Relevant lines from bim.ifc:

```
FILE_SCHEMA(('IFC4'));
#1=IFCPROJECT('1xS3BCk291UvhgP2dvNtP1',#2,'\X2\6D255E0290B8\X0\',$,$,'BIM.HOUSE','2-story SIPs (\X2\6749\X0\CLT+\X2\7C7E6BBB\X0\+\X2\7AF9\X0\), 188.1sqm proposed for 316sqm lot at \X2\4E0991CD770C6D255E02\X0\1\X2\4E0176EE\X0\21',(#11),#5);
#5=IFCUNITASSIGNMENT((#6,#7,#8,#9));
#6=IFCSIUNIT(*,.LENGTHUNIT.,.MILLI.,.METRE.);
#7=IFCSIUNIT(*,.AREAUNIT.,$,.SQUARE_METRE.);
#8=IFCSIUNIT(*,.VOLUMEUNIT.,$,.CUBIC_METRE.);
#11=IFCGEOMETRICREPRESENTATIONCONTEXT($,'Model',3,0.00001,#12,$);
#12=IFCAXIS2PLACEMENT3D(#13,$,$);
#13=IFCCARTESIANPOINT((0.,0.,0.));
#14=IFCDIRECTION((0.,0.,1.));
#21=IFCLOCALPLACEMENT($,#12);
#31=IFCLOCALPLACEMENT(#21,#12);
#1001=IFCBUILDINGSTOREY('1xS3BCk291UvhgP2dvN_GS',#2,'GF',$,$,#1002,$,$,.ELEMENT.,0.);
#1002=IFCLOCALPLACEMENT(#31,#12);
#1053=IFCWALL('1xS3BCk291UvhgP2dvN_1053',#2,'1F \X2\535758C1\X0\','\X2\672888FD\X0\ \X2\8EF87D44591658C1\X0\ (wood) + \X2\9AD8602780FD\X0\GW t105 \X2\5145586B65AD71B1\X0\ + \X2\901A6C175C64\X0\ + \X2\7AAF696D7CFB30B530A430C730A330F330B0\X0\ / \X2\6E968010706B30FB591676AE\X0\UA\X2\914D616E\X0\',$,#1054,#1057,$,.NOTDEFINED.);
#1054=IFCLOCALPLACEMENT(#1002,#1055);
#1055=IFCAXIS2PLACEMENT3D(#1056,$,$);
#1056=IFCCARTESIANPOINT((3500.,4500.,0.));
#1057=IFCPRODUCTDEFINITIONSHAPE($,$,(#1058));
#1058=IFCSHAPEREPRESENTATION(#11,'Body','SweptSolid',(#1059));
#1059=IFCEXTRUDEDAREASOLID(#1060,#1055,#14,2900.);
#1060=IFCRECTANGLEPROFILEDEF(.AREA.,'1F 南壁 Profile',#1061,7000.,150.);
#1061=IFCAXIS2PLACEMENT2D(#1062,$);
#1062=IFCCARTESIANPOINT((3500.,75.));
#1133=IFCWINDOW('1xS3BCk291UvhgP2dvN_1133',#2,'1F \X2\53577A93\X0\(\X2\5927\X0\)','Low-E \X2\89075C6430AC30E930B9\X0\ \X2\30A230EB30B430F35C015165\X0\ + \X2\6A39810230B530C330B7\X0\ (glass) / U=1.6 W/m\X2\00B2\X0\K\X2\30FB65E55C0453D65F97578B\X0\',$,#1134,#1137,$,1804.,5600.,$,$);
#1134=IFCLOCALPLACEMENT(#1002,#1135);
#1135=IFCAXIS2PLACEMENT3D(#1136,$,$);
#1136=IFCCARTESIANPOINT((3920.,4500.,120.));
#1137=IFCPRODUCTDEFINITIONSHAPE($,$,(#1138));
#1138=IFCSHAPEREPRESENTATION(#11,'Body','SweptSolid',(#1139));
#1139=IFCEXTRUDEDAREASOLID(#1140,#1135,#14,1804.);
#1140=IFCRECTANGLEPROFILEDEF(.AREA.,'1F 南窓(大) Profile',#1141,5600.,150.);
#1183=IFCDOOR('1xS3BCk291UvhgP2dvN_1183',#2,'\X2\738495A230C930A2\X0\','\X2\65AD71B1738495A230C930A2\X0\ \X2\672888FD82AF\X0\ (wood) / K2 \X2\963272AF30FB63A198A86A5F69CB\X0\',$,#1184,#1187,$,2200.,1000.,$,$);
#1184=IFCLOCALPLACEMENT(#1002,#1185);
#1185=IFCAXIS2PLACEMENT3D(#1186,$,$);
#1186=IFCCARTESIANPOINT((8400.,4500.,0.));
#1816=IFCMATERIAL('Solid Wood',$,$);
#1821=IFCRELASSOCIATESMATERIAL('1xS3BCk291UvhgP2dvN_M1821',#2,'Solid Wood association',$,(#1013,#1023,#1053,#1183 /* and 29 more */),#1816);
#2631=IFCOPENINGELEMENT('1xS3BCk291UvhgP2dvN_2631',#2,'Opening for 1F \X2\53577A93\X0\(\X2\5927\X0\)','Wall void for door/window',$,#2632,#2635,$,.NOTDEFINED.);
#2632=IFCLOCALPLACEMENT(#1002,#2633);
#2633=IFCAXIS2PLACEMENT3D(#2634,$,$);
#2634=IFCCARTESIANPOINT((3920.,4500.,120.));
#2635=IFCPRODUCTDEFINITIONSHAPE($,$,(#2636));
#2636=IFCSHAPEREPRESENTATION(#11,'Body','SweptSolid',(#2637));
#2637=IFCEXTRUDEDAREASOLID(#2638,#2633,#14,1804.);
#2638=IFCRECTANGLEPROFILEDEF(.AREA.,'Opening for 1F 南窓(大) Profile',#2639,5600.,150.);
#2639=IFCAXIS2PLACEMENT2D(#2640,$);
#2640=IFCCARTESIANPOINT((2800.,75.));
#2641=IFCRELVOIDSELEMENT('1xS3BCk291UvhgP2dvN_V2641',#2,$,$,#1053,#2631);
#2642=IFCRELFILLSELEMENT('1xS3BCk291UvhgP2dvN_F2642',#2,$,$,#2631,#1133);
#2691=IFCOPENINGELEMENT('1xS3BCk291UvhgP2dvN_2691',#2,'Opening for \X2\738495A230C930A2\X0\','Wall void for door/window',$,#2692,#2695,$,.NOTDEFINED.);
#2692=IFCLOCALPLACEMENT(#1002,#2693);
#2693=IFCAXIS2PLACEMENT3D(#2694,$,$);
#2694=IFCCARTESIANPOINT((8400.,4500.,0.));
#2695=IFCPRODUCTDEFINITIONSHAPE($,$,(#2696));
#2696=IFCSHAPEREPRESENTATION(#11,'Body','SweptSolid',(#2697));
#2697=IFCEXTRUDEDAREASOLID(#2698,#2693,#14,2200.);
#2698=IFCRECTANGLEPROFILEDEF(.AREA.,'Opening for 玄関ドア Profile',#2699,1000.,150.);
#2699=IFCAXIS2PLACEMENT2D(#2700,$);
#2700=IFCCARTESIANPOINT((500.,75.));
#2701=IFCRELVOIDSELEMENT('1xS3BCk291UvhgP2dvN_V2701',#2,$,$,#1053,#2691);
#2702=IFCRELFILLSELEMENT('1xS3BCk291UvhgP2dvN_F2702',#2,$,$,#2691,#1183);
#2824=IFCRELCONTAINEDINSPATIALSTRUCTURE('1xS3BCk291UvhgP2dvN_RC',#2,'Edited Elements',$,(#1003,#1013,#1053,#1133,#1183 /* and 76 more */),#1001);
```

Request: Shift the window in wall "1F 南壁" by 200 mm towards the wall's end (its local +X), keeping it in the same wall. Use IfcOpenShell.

```python
import ifcopenshell
import ifcopenshell.api.geometry
import ifcopenshell.util.placement

model = ifcopenshell.open("bim.ifc")

window = model.by_guid("1xS3BCk291UvhgP2dvN_1133")
opening = window.FillsVoids[0].RelatingOpeningElement
wall = opening.VoidsElements[0].RelatingBuildingElement

wall_matrix = ifcopenshell.util.placement.get_local_placement(wall.ObjectPlacement)
shift = wall_matrix[:3, 0] * 200.0
before = ifcopenshell.util.placement.get_local_placement(window.ObjectPlacement)[:3, 3].copy()

# The window is not placed relative to its opening, so move both.
for product in (opening, window):
    matrix = ifcopenshell.util.placement.get_local_placement(product.ObjectPlacement)
    matrix[:3, 3] += shift
    ifcopenshell.api.geometry.edit_object_placement(model, product=product, matrix=matrix, is_si=False)

after = ifcopenshell.util.placement.get_local_placement(window.ObjectPlacement)[:3, 3]
print("window moved by", (after - before).round(3) + 0.0)

model.write("bim_v2.ifc")
```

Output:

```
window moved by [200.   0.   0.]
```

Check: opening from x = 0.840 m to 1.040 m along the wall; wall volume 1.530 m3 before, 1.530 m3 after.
